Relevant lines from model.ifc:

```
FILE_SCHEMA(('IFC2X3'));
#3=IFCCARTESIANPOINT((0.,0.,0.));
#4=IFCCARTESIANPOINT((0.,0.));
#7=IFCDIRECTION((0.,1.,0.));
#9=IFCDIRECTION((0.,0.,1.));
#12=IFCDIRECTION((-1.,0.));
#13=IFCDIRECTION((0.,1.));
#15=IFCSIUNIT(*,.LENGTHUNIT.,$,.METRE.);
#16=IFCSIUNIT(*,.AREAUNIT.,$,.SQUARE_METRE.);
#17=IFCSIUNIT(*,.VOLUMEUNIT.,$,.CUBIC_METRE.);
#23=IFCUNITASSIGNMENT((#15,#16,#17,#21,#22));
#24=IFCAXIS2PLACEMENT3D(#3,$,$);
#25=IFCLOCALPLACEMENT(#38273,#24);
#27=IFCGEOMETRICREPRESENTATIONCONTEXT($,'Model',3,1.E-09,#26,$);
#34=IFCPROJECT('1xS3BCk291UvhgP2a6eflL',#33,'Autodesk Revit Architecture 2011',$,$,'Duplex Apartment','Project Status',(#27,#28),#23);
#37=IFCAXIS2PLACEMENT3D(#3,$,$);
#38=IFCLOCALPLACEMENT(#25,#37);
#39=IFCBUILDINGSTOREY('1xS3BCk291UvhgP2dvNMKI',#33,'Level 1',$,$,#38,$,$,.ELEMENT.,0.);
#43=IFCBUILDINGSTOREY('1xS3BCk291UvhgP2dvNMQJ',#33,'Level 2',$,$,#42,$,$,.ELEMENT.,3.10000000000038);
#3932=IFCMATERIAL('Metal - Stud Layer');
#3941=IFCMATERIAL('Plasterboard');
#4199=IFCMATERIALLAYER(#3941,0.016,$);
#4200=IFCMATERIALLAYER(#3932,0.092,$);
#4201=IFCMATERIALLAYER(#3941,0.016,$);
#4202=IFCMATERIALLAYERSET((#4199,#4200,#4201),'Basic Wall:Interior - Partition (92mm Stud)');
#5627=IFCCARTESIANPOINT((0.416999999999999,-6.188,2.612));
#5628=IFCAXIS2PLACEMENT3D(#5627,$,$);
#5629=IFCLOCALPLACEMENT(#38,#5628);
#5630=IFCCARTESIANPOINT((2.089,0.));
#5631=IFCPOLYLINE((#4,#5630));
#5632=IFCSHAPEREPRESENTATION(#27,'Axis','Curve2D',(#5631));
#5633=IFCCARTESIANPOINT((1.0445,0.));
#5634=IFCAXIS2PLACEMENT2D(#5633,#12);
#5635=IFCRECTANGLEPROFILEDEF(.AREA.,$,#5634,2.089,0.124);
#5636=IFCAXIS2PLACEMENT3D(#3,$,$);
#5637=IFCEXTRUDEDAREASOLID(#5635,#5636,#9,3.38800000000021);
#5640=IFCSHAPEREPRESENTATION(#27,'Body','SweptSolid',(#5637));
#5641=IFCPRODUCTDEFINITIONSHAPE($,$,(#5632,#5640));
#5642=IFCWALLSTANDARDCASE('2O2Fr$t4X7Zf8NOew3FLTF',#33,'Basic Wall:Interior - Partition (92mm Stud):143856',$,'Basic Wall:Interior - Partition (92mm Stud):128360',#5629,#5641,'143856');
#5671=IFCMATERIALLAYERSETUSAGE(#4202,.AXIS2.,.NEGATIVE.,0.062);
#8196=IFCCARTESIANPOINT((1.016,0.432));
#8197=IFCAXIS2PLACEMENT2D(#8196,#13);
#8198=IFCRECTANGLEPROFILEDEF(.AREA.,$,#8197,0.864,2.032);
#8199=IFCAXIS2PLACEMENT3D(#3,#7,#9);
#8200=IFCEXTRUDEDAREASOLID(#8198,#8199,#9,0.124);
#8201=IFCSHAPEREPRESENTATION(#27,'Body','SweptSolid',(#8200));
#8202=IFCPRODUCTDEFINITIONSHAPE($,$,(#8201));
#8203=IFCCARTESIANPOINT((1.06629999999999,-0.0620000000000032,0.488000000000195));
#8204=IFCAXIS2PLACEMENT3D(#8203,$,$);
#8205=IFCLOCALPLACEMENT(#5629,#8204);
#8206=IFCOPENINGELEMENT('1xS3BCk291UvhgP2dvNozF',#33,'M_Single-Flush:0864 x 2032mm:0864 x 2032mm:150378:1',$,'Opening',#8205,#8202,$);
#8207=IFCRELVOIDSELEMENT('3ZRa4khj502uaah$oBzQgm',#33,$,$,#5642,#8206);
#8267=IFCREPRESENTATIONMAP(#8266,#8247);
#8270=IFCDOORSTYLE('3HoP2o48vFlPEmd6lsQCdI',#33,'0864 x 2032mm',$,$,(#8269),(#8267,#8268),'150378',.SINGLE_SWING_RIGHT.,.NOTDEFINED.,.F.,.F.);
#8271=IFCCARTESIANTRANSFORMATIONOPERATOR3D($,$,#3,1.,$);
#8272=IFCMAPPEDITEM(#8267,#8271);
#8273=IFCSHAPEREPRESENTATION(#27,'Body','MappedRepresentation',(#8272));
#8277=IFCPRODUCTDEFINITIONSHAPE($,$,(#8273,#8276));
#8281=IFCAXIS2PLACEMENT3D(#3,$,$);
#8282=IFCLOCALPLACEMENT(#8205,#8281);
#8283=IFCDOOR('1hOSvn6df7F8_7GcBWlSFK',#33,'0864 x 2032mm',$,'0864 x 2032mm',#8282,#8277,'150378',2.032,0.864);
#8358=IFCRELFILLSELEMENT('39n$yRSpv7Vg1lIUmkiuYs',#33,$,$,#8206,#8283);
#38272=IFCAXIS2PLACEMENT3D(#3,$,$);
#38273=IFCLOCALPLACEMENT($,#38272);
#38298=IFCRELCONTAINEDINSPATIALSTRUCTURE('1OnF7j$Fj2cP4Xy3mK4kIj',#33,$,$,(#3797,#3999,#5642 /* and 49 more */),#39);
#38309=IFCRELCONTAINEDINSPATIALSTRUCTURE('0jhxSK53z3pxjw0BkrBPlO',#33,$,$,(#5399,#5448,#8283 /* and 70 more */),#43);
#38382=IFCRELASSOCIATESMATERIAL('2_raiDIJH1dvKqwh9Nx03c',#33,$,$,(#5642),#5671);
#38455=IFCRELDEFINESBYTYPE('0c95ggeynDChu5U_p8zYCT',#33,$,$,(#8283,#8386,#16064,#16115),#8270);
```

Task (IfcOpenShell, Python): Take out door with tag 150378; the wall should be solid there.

```python
import ifcopenshell
import ifcopenshell.api.feature
import ifcopenshell.api.root
import ifcopenshell.geom
import ifcopenshell.util.shape

model = ifcopenshell.open("model.ifc")
settings = ifcopenshell.geom.settings()


def volume(element):
    """Net volume in cubic metres, openings subtracted."""
    shape = ifcopenshell.geom.create_shape(settings, element)
    return ifcopenshell.util.shape.get_volume(shape.geometry)


door = model.by_id(8283)
opening = door.FillsVoids[0].RelatingOpeningElement
wall = opening.VoidsElements[0].RelatingBuildingElement
before = volume(wall)

ifcopenshell.api.root.remove_product(model, product=door)
ifcopenshell.api.feature.remove_feature(model, feature=opening)

after = volume(wall)

print(f"wall volume {before:.3f} -> {after:.3f} m3")

model.write("model_edited.ifc")
```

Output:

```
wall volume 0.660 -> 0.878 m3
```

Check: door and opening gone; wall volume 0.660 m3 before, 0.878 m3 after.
